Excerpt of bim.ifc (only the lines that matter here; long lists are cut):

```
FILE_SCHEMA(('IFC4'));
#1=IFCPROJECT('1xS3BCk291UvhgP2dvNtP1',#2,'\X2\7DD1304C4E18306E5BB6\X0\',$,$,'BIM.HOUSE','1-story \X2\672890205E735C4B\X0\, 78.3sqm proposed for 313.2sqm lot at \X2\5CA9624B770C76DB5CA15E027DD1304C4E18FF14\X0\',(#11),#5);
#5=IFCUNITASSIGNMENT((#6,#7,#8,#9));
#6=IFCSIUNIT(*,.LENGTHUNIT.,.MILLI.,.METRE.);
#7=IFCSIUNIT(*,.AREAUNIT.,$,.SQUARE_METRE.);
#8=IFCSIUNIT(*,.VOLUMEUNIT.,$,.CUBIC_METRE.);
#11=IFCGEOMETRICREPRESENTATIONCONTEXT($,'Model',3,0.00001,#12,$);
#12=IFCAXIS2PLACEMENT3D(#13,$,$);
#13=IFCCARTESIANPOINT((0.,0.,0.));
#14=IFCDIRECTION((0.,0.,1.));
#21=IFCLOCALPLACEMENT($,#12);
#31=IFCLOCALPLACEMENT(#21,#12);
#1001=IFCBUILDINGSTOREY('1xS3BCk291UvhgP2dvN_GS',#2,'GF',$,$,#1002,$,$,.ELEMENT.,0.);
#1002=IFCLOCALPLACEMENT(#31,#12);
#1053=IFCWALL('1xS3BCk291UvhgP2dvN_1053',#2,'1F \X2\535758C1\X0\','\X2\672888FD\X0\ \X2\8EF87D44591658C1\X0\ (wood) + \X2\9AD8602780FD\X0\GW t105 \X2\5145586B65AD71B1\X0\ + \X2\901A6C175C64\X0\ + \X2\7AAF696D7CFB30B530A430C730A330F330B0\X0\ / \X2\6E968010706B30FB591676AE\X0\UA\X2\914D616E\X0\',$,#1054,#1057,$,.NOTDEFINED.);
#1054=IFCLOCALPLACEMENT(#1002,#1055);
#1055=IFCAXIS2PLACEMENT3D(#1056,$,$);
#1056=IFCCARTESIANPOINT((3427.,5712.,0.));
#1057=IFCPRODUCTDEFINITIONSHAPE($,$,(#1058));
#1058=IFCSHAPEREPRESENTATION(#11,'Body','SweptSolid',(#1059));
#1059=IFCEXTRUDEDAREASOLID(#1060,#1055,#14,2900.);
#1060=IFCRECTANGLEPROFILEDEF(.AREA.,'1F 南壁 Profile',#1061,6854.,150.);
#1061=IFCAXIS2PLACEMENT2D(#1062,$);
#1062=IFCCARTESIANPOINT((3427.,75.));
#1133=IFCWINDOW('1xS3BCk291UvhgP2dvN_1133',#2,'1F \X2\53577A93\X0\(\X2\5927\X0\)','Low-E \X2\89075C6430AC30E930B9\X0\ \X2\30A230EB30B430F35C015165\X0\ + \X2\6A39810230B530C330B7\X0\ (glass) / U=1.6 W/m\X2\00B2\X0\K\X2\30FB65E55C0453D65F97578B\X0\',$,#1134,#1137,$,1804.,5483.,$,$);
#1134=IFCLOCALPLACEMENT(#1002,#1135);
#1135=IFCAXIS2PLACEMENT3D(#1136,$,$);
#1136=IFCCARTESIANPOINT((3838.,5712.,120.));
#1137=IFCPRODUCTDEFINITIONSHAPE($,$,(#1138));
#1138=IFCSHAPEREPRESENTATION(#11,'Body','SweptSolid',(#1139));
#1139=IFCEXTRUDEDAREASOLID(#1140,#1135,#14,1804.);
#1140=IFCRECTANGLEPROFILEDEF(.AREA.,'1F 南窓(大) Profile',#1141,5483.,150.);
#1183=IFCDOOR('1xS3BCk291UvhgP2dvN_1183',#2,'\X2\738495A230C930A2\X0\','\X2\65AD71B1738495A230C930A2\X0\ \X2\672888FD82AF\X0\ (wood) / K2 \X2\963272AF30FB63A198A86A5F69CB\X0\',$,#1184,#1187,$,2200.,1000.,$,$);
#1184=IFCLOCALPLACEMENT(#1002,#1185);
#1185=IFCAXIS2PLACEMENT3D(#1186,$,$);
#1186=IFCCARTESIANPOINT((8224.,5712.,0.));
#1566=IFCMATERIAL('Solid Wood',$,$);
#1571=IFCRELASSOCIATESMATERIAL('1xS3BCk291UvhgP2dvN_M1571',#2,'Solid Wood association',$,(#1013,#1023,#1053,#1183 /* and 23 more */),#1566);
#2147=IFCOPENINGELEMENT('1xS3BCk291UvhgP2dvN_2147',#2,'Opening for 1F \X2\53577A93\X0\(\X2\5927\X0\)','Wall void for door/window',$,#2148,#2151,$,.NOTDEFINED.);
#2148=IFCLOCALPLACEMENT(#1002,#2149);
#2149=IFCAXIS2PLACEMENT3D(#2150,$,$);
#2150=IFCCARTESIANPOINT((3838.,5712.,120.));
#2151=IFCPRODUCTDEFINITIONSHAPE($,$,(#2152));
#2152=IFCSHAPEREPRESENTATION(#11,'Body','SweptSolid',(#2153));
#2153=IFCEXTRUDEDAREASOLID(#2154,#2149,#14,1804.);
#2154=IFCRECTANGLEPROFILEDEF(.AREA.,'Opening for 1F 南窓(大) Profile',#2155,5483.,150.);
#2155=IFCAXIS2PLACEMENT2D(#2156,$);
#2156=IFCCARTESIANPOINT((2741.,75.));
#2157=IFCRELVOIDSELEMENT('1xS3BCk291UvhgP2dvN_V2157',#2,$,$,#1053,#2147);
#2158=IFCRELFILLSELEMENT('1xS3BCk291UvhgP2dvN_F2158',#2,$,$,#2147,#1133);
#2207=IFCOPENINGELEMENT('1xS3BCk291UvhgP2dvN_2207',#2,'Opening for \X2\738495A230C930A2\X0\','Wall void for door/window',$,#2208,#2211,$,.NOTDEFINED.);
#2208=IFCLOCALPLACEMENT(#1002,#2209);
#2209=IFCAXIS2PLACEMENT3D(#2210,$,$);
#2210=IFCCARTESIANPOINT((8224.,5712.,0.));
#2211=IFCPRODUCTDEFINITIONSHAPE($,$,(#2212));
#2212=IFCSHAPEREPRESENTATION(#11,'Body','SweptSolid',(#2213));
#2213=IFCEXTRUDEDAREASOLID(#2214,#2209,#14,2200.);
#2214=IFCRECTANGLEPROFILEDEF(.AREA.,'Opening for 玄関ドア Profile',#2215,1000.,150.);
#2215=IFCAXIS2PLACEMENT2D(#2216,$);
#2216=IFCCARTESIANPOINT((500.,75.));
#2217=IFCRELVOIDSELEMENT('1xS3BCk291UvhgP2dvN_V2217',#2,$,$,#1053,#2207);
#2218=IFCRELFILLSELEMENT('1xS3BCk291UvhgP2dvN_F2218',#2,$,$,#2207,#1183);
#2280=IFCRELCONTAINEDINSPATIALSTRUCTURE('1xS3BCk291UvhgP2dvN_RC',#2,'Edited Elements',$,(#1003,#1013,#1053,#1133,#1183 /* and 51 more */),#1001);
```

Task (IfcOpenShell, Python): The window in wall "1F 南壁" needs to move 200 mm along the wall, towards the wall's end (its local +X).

```python
import ifcopenshell
import ifcopenshell.api.geometry
import ifcopenshell.util.placement
import ifcopenshell.util.unit

model = ifcopenshell.open("bim.ifc")
unit_scale = ifcopenshell.util.unit.calculate_unit_scale(model)

window = model.by_id(1133)
opening = window.FillsVoids[0].RelatingOpeningElement
wall = opening.VoidsElements[0].RelatingBuildingElement

wall_matrix = ifcopenshell.util.placement.get_local_placement(wall.ObjectPlacement)
shift = wall_matrix[:3, 0] * 0.2 / unit_scale
before = ifcopenshell.util.placement.get_local_placement(window.ObjectPlacement)[:3, 3].copy()

# The window is not placed relative to its opening, so move both.
for product in (opening, window):
    matrix = ifcopenshell.util.placement.get_local_placement(product.ObjectPlacement)
    matrix[:3, 3] += shift
    ifcopenshell.api.geometry.edit_object_placement(model, product=product, matrix=matrix, is_si=False)

after = ifcopenshell.util.placement.get_local_placement(window.ObjectPlacement)[:3, 3]
print("window moved by", (after - before).round(3) + 0.0)

model.write("bim_v2.ifc")
```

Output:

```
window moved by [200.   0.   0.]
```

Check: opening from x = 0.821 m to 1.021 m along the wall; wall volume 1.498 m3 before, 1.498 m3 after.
